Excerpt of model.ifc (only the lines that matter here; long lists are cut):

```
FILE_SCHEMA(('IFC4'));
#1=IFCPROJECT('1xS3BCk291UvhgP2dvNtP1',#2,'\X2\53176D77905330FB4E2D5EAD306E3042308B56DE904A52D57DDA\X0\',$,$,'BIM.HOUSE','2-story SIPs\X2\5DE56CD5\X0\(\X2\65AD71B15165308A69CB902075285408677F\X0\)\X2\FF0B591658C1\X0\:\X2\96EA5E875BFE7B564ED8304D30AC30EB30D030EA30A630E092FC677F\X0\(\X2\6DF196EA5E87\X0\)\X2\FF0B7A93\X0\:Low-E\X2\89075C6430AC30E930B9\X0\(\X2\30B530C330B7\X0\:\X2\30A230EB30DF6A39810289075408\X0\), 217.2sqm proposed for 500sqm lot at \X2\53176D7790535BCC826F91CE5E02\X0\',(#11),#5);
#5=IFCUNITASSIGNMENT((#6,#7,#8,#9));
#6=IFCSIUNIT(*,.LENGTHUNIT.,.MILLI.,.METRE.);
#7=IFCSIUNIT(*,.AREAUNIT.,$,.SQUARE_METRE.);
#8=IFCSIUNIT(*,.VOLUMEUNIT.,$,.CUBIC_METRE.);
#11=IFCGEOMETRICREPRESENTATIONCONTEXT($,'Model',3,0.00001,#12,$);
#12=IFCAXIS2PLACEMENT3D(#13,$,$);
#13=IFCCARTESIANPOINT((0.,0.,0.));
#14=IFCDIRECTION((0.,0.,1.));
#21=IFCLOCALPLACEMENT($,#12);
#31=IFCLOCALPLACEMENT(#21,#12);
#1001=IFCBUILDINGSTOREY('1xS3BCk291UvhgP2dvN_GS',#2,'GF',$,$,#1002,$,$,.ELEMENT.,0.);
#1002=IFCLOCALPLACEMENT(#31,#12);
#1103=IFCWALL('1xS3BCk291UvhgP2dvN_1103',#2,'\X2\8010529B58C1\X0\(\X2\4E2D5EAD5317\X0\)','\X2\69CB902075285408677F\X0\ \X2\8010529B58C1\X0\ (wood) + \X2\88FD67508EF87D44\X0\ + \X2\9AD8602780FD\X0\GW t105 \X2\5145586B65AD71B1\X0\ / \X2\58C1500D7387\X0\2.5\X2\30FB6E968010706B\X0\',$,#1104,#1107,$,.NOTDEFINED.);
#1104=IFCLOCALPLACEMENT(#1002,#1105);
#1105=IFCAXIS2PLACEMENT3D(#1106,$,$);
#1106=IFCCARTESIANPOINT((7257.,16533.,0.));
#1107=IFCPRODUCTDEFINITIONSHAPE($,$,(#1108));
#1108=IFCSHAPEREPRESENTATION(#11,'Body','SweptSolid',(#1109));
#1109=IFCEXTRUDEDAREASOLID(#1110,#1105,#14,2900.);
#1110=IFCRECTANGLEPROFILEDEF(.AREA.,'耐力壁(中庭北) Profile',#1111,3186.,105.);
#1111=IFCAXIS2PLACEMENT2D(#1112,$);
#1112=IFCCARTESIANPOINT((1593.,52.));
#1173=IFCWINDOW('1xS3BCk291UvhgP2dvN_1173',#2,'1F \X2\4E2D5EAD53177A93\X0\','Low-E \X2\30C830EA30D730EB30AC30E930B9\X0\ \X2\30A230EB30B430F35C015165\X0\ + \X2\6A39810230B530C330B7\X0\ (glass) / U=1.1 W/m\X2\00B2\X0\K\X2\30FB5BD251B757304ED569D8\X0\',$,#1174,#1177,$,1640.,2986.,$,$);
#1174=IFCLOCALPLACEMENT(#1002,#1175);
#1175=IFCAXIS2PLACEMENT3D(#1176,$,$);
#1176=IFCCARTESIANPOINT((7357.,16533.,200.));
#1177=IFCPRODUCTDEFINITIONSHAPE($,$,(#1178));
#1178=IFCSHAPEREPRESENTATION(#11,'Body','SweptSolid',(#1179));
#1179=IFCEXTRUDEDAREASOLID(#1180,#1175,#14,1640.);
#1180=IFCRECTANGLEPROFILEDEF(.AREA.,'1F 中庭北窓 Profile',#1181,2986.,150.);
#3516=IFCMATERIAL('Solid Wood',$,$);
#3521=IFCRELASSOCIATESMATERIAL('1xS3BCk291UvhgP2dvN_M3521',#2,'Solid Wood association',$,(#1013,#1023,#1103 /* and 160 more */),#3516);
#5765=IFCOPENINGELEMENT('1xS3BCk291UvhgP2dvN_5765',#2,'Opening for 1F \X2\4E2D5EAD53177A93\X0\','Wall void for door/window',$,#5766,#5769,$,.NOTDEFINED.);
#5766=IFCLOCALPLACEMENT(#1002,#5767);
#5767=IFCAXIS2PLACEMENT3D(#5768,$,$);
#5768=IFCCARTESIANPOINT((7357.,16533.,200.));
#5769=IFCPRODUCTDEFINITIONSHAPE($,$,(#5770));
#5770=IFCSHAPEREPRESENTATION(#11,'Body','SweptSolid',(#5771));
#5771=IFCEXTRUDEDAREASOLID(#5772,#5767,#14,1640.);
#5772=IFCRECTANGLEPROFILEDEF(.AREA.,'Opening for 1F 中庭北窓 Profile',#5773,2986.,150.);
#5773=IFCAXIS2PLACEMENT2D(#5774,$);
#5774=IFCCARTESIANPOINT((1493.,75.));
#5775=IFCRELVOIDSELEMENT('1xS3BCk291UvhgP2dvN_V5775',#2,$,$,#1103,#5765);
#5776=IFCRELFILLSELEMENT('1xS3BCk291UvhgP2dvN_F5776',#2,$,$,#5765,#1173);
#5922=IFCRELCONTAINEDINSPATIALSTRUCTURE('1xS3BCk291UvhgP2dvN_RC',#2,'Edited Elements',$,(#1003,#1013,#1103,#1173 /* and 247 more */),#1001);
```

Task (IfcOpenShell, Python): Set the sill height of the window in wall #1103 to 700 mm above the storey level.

```python
import numpy as np
import ifcopenshell
import ifcopenshell.api.geometry
import ifcopenshell.geom
import ifcopenshell.util.element
import ifcopenshell.util.placement
import ifcopenshell.util.shape
import ifcopenshell.util.unit

model = ifcopenshell.open("model.ifc")
unit_scale = ifcopenshell.util.unit.calculate_unit_scale(model)

window = model.by_id(1173)
opening = window.FillsVoids[0].RelatingOpeningElement
storey = ifcopenshell.util.element.get_container(window, ifc_class="IfcBuildingStorey")
level = ifcopenshell.util.placement.get_local_placement(storey.ObjectPlacement)[2, 3]

# The opening's origin need not be at the sill, so measure its lowest point.
shape = ifcopenshell.geom.create_shape(ifcopenshell.geom.settings(), opening)
bottom = ifcopenshell.util.shape.get_shape_bottom_elevation(shape, shape.geometry) / unit_scale
dz = level + 0.7 / unit_scale - bottom

shift = np.array([0.0, 0.0, dz])
# The window is not placed relative to its opening, so move both.
for product in (opening, window):
    matrix = ifcopenshell.util.placement.get_local_placement(product.ObjectPlacement)
    matrix[:3, 3] += shift
    ifcopenshell.api.geometry.edit_object_placement(model, product=product, matrix=matrix, is_si=False)

print(f"moved by {dz * unit_scale:+.3f} m")

model.write("model_updated.ifc")
```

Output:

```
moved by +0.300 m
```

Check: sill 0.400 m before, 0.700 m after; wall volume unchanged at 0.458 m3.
